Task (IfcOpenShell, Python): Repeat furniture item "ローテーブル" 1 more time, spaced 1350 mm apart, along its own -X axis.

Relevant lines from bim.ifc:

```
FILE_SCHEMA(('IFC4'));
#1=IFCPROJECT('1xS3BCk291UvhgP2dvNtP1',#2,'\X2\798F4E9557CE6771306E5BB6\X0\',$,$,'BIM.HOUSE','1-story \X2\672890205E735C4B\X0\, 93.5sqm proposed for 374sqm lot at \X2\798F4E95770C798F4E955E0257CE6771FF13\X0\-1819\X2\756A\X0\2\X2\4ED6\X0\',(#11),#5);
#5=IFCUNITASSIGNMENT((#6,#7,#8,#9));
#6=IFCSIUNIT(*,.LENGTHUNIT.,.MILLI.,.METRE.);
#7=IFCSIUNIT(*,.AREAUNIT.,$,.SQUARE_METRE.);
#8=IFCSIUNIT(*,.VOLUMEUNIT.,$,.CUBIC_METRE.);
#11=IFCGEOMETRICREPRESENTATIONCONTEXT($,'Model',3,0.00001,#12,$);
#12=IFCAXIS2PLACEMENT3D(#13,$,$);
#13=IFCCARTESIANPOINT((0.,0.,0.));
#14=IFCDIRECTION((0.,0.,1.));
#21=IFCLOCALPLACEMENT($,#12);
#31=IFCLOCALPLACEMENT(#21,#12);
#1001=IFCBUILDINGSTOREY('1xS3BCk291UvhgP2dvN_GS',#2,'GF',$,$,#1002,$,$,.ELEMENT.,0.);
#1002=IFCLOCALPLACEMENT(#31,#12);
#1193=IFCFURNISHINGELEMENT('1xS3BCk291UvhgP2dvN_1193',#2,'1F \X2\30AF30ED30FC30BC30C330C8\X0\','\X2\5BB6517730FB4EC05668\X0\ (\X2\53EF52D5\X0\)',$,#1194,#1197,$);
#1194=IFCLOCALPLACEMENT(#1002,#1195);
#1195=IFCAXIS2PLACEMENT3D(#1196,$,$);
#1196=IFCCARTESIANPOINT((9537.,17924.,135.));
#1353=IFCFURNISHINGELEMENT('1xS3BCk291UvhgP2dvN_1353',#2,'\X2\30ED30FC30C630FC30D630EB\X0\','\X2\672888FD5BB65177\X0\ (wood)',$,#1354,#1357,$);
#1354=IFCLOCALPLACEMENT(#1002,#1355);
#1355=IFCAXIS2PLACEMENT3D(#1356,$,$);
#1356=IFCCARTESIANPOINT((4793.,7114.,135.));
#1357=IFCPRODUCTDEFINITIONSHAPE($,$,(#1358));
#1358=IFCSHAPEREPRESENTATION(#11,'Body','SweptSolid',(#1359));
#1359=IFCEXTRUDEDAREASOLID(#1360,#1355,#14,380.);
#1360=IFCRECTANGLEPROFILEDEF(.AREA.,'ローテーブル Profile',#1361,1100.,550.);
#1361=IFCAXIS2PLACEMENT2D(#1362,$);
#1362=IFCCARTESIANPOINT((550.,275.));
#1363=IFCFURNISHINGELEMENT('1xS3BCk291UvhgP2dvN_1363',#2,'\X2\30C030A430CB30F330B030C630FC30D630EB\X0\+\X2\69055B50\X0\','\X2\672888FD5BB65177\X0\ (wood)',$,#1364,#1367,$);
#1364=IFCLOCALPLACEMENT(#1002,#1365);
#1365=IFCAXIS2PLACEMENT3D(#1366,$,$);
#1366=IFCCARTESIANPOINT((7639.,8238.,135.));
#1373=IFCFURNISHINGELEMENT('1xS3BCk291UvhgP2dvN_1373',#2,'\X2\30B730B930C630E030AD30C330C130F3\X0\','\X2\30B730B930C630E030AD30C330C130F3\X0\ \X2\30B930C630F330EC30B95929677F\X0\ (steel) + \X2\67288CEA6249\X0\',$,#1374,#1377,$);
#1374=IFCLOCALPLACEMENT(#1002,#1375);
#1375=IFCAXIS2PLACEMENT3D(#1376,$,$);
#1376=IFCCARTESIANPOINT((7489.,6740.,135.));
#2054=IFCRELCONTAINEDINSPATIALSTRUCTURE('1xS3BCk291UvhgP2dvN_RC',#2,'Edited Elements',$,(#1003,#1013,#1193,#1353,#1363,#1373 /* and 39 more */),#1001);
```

```python
import ifcopenshell
import ifcopenshell.api.geometry
import ifcopenshell.api.root
import ifcopenshell.util.element
import ifcopenshell.util.placement
import ifcopenshell.util.unit

model = ifcopenshell.open("bim.ifc")
unit_scale = ifcopenshell.util.unit.calculate_unit_scale(model)


def reuse_history(source, copy):
    """copy_class also copies each property set's owner history, people and application; keep the originals."""
    for rel in copy.IsDefinedBy:
        if rel.is_a("IfcRelDefinesByProperties") and (history := rel.RelatingPropertyDefinition.OwnerHistory):
            rel.RelatingPropertyDefinition.OwnerHistory = source.OwnerHistory
            ifcopenshell.util.element.remove_deep2(model, history)


source = model.by_id(1353)
base = ifcopenshell.util.placement.get_local_placement(source.ObjectPlacement)
step = -base[:3, 0] * 1.35 / unit_scale

for i in range(1, 2):
    copy = ifcopenshell.api.root.copy_class(model, product=source)
    copy.Representation = ifcopenshell.util.element.copy_deep(
        model, source.Representation, exclude=["IfcGeometricRepresentationContext", "IfcRepresentationMap"]
    )
    reuse_history(source, copy)
    matrix = base.copy()
    matrix[:3, 3] += i * step
    print("added at", matrix[:3, 3].round(3) + 0.0)
    ifcopenshell.api.geometry.edit_object_placement(model, product=copy, matrix=matrix, is_si=False)

model.write("bim_v2.ifc")
```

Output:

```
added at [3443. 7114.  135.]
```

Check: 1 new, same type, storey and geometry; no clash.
